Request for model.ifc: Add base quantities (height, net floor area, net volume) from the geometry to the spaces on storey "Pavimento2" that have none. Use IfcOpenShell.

First a look at what the model holds.

```python
import ifcopenshell
import ifcopenshell.util.element
import ifcopenshell.util.unit

model = ifcopenshell.open("model.ifc")
print(model.schema)
for unit_type in ("LENGTHUNIT", "AREAUNIT", "VOLUMEUNIT"):
    print(unit_type, ifcopenshell.util.unit.calculate_unit_scale(model, unit_type))
storey = next(s for s in model.by_type("IfcBuildingStorey") if s.Name == "Pavimento2")
spaces = [e for e in ifcopenshell.util.element.get_decomposition(storey) if e.is_a("IfcSpace")]
for e in sorted(spaces, key=lambda e: e.id()):
    print(e.id(), e.is_a(), e.Name, list(ifcopenshell.util.element.get_psets(e, qtos_only=True)), sep=" | ")
```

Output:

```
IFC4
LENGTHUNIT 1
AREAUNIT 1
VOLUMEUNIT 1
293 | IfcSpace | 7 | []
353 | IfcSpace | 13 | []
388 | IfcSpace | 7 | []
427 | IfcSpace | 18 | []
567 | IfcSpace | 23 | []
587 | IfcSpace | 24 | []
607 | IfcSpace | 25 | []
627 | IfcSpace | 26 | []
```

```python
import ifcopenshell
import ifcopenshell.api.pset
import ifcopenshell.geom
import ifcopenshell.util.element
import ifcopenshell.util.shape
import ifcopenshell.util.unit

model = ifcopenshell.open("model.ifc")
unit_scale = ifcopenshell.util.unit.calculate_unit_scale(model)
area_scale = ifcopenshell.util.unit.calculate_unit_scale(model, "AREAUNIT")
volume_scale = ifcopenshell.util.unit.calculate_unit_scale(model, "VOLUMEUNIT")
settings = ifcopenshell.geom.settings()

storey = next(s for s in model.by_type("IfcBuildingStorey") if s.Name == "Pavimento2")
spaces = [e for e in ifcopenshell.util.element.get_decomposition(storey) if e.is_a("IfcSpace")]

for e in sorted(spaces, key=lambda e: e.id()):
    if ifcopenshell.util.element.get_psets(e, qtos_only=True, should_inherit=False):
        continue
    # Geometry comes back in metres, in the element's own axes.
    shape = ifcopenshell.geom.create_shape(settings, e)
    values = {
        "Height": ifcopenshell.util.shape.get_z(shape.geometry) / unit_scale,
        "NetFloorArea": ifcopenshell.util.shape.get_footprint_area(shape.geometry) / area_scale,
        "NetVolume": ifcopenshell.util.shape.get_volume(shape.geometry) / volume_scale,
    }
    qto = ifcopenshell.api.pset.add_qto(model, product=e, name="Qto_SpaceBaseQuantities")
    ifcopenshell.api.pset.edit_qto(model, qto=qto, properties=values)
    print(e.id(), {k: round(v, 3) for k, v in values.items()})

model.write("model_v2.ifc")
```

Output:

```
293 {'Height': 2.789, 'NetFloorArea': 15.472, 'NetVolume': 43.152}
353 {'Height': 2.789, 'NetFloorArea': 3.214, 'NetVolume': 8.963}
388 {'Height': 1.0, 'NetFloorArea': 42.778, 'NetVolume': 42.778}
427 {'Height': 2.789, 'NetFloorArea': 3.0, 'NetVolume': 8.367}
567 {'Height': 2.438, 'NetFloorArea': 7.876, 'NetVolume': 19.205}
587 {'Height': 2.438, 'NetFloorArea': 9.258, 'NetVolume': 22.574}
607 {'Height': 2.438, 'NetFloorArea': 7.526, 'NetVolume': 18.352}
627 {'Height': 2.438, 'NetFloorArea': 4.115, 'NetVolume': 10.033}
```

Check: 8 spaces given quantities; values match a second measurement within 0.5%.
